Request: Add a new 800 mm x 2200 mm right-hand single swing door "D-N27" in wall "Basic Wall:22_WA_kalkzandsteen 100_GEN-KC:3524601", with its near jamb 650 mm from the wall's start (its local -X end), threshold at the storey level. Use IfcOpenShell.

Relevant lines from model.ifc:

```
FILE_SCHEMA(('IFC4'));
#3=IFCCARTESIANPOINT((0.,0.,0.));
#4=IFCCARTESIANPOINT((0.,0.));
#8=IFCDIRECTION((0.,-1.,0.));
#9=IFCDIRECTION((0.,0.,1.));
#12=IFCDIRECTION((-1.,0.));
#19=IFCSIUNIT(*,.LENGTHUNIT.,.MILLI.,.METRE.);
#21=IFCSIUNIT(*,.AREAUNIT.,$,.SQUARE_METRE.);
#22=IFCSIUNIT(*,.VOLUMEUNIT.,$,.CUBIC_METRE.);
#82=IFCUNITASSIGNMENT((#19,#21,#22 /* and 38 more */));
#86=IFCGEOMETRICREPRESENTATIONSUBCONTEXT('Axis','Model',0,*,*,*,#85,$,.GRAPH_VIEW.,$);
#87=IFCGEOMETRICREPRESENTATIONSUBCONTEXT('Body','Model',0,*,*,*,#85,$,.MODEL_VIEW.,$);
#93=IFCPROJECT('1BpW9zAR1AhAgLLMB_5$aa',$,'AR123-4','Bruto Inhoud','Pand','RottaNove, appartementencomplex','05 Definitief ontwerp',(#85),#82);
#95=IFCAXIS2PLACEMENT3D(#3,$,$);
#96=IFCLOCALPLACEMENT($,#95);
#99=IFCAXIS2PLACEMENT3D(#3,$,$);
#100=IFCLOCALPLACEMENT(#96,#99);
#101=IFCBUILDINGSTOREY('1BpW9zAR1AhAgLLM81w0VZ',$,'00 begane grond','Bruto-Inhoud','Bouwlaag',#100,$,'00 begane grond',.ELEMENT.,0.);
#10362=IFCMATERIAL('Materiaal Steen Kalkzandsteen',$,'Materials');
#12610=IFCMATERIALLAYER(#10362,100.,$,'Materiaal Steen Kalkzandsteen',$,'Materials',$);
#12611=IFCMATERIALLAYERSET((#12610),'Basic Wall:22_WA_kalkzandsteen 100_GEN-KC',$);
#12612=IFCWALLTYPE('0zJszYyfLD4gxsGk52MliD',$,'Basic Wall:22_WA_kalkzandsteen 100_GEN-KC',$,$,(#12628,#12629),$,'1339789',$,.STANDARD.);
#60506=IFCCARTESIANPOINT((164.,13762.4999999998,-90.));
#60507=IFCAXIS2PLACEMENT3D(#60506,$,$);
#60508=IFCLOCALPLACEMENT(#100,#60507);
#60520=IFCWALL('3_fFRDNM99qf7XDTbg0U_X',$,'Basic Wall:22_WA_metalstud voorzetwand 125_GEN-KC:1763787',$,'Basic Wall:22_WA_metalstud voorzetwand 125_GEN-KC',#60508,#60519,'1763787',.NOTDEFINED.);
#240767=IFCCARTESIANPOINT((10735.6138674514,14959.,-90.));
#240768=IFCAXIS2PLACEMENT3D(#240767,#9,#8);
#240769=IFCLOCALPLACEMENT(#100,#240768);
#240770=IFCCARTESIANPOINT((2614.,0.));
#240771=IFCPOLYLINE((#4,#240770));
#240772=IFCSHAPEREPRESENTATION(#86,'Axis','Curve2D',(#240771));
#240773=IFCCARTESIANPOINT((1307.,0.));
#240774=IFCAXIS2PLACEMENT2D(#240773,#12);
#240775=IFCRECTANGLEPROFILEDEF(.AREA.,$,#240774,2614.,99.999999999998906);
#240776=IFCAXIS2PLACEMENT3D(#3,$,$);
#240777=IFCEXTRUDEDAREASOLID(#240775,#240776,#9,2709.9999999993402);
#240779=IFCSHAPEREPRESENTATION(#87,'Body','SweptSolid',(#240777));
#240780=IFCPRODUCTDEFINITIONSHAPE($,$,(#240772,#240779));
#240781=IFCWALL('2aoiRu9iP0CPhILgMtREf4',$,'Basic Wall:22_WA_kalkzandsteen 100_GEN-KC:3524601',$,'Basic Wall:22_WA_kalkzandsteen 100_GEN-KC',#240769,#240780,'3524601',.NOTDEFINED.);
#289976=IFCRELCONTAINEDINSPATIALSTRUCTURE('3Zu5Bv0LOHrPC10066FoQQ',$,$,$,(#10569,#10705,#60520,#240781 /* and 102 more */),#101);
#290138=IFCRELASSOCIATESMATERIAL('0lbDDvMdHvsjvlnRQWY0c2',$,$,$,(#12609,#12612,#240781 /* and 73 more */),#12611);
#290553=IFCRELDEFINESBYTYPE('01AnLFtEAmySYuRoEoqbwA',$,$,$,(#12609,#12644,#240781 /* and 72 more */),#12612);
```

```python
import numpy as np
import ifcopenshell
import ifcopenshell.api.feature
import ifcopenshell.api.geometry
import ifcopenshell.api.root
import ifcopenshell.api.spatial
import ifcopenshell.geom
import ifcopenshell.util.element
import ifcopenshell.util.placement
import ifcopenshell.util.representation
import ifcopenshell.util.shape
import ifcopenshell.util.unit

model = ifcopenshell.open("model.ifc")
unit_scale = ifcopenshell.util.unit.calculate_unit_scale(model)
settings = ifcopenshell.geom.settings()


def volume(element):
    """Net volume in cubic metres, openings subtracted."""
    shape = ifcopenshell.geom.create_shape(settings, element)
    return ifcopenshell.util.shape.get_volume(shape.geometry)


wall = model.by_guid("2aoiRu9iP0CPhILgMtREf4")
storey = ifcopenshell.util.element.get_container(wall, ifc_class="IfcBuildingStorey")
context = ifcopenshell.util.representation.get_context(model, "Model", "Body", "MODEL_VIEW")
before = volume(wall)

width, height, from_end, sill = 0.8, 2.2, 0.65, 0.0  # metres

# The wall runs along its own X axis, and the end named is its -X end.
wall_shape = ifcopenshell.geom.create_shape(settings, wall)
x, y, z = ifcopenshell.util.shape.get_vertices(wall_shape.geometry).T
start = x.min() + from_end
face, thickness = float(y.min()), float(y.max() - y.min())
wall_matrix = ifcopenshell.util.placement.get_local_placement(wall.ObjectPlacement)
level = ifcopenshell.util.placement.get_local_placement(storey.ObjectPlacement)[2, 3]


def in_wall(x, y):
    """Placement at x, y metres in the wall's axes, at sill height."""
    matrix = wall_matrix.copy()
    matrix[:, 3] = wall_matrix @ np.array([x / unit_scale, y / unit_scale, 0.0, 1.0])
    matrix[2, 3] = level + sill / unit_scale
    return matrix


# Opening: a box that overshoots both wall faces by 50 mm.
opening = ifcopenshell.api.root.create_entity(model, ifc_class="IfcOpeningElement", predefined_type="OPENING")
box = ifcopenshell.api.geometry.add_wall_representation(
    model, context=context, length=width, height=height, thickness=thickness + 0.1
)
ifcopenshell.api.geometry.assign_representation(model, product=opening, representation=box)
ifcopenshell.api.geometry.edit_object_placement(model, product=opening, matrix=in_wall(start, face - 0.05), is_si=False)
ifcopenshell.api.feature.add_feature(model, feature=opening, element=wall)

door = ifcopenshell.api.root.create_entity(model, ifc_class="IfcDoor", name="D-N27", predefined_type="DOOR")
door.OverallWidth, door.OverallHeight = width / unit_scale, height / unit_scale
door.OperationType = "SINGLE_SWING_RIGHT"
body = ifcopenshell.api.geometry.add_door_representation(
    model,
    context=context,
    overall_width=door.OverallWidth,
    overall_height=door.OverallHeight,
    operation_type="SINGLE_SWING_RIGHT",
    lining_properties={"LiningDepth": thickness / unit_scale, "ThresholdDepth": thickness / unit_scale},
)
ifcopenshell.api.geometry.assign_representation(model, product=door, representation=body)
ifcopenshell.api.spatial.assign_container(model, products=[door], relating_structure=storey)
ifcopenshell.api.feature.add_filling(model, opening=opening, element=door)

# The lining spans the wall, so the door starts at the wall face.
ifcopenshell.api.geometry.edit_object_placement(model, product=door, matrix=in_wall(start, face), is_si=False)

after = volume(wall)

print(f"wall volume {before:.3f} -> {after:.3f} m3")

model.write("model_rev.ifc")
```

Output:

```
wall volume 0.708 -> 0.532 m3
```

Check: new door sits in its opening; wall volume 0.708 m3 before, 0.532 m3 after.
